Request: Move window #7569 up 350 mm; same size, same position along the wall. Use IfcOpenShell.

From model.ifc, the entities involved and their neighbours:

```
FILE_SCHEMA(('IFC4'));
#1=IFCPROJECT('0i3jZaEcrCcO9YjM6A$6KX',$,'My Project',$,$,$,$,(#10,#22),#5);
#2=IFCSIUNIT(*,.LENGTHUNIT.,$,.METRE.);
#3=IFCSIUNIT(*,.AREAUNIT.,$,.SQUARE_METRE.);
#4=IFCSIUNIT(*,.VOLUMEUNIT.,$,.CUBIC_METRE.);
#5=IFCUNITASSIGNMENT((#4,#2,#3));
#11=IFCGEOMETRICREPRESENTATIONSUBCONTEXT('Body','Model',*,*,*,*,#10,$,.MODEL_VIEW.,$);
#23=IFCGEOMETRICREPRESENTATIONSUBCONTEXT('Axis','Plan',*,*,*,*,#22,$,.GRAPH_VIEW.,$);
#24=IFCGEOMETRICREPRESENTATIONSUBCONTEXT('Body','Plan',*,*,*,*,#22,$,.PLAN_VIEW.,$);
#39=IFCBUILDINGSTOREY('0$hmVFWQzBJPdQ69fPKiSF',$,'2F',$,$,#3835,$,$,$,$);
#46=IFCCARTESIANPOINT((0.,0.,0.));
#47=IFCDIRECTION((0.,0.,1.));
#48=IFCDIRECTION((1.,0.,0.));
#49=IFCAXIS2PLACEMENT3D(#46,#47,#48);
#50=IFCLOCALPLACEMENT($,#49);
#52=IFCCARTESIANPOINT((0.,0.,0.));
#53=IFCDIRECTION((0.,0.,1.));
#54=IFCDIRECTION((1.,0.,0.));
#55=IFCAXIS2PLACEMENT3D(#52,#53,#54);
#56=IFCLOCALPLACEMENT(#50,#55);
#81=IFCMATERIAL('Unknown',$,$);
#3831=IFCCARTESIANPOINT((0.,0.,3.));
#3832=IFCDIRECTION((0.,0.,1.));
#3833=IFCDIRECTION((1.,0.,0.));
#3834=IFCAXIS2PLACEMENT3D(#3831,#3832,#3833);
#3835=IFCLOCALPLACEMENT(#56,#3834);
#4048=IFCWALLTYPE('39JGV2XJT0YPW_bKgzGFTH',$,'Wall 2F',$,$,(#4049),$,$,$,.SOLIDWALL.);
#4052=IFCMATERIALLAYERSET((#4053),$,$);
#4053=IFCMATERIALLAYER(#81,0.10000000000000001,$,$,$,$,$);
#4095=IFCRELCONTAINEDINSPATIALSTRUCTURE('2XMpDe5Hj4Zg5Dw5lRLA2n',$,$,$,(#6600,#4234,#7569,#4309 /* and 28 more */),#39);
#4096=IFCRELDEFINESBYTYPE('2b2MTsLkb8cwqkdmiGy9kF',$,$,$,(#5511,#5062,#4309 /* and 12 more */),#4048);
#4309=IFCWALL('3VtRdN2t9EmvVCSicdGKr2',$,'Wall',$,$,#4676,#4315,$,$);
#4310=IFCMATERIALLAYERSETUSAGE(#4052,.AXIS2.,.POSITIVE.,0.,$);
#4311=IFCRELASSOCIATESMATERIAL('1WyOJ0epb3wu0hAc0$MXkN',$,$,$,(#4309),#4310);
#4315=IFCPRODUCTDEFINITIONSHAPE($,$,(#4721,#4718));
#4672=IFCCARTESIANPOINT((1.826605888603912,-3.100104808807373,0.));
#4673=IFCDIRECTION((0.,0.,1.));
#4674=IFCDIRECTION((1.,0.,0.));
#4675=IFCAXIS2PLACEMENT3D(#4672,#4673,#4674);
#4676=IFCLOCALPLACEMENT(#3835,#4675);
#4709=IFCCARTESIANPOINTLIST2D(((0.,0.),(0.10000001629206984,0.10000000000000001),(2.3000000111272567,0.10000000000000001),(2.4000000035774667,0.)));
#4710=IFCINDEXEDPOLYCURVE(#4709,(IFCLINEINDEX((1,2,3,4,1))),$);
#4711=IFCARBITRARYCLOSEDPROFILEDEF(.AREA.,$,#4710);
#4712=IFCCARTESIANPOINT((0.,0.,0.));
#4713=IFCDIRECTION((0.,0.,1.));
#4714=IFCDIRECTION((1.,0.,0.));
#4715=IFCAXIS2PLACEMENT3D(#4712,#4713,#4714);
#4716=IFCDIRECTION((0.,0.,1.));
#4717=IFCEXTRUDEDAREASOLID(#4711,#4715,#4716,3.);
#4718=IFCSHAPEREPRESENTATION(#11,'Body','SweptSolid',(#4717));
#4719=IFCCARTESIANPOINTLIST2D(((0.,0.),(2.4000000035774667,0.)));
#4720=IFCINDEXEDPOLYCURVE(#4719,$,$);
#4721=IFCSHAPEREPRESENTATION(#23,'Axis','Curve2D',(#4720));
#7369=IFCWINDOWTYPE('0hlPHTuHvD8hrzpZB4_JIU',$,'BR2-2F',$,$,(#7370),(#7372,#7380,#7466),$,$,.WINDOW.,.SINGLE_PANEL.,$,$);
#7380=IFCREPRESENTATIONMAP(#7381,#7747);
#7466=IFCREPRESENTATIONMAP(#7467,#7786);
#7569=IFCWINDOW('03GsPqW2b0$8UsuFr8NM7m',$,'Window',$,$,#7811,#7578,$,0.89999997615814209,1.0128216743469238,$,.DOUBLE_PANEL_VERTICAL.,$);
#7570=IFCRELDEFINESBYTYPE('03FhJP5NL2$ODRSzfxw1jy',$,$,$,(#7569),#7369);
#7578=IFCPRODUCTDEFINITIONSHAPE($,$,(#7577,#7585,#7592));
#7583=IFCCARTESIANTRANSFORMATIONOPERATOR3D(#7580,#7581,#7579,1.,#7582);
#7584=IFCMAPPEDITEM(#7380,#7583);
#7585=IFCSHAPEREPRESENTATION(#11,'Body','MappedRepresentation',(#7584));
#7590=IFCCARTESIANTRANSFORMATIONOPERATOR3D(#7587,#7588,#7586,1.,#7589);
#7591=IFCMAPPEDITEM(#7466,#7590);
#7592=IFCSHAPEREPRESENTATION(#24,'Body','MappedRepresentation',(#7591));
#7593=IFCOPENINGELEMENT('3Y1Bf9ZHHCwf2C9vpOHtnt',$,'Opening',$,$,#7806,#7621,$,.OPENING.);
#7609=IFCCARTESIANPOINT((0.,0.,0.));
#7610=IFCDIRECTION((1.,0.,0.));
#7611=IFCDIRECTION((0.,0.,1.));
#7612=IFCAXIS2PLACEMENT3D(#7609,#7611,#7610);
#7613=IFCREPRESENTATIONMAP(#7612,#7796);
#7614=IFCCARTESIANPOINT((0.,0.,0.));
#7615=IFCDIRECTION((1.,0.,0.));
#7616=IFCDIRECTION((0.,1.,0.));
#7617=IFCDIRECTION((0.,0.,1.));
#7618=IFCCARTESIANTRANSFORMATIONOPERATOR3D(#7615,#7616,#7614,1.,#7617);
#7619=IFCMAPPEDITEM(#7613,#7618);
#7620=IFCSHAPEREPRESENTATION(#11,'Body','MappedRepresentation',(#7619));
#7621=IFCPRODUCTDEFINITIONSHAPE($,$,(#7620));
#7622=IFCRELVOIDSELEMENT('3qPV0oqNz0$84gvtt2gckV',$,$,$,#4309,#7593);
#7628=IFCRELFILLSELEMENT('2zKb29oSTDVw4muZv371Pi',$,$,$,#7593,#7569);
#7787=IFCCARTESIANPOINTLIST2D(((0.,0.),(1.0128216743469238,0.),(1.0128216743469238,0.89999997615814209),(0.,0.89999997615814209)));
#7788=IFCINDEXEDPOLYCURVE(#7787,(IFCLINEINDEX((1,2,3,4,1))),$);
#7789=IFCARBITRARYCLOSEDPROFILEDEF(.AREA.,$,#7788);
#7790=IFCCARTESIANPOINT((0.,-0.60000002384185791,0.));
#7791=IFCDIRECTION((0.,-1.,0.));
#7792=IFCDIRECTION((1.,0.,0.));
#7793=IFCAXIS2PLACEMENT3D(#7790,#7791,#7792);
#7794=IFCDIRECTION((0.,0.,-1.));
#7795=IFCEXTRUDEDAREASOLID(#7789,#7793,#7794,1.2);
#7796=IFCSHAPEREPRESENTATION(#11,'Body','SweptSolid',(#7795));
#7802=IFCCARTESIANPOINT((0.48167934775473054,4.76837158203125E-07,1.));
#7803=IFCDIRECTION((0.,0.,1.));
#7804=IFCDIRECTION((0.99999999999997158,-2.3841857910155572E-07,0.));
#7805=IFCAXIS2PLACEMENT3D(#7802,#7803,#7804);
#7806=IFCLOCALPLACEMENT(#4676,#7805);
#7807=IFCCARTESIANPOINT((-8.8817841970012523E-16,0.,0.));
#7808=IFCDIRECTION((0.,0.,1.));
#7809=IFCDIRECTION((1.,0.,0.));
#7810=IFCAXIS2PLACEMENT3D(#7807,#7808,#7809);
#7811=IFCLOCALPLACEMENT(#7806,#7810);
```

```python
import numpy as np
import ifcopenshell
import ifcopenshell.api.geometry
import ifcopenshell.util.placement
import ifcopenshell.util.unit

model = ifcopenshell.open("model.ifc")
unit_scale = ifcopenshell.util.unit.calculate_unit_scale(model)

window = model.by_guid("03GsPqW2b0$8UsuFr8NM7m")
opening = window.FillsVoids[0].RelatingOpeningElement
dz = 0.35 / unit_scale

shift = np.array([0.0, 0.0, dz])
# The window is placed relative to its opening, so it follows when the opening moves.
matrix = ifcopenshell.util.placement.get_local_placement(opening.ObjectPlacement)
matrix[:3, 3] += shift
ifcopenshell.api.geometry.edit_object_placement(
    model, product=opening, matrix=matrix, is_si=False, should_transform_children=True
)

print(f"moved by {dz * unit_scale:+.3f} m")

model.write("model_rev.ifc")
```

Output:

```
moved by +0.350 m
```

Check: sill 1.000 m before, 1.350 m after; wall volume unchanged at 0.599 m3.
